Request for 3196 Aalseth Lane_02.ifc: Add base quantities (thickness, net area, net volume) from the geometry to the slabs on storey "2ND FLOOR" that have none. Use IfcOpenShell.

First a look at what the model holds.

```python
import ifcopenshell
import ifcopenshell.util.element
import ifcopenshell.util.unit

model = ifcopenshell.open("3196 Aalseth Lane_02.ifc")
print(model.schema)
for unit_type in ("LENGTHUNIT", "AREAUNIT", "VOLUMEUNIT"):
    print(unit_type, ifcopenshell.util.unit.calculate_unit_scale(model, unit_type))
storey = next(s for s in model.by_type("IfcBuildingStorey") if s.Name == "2ND FLOOR")
slabs = [e for e in ifcopenshell.util.element.get_decomposition(storey) if e.is_a("IfcSlab")]
for e in sorted(slabs, key=lambda e: e.id()):
    print(e.id(), e.is_a(), e.Name, list(ifcopenshell.util.element.get_psets(e, qtos_only=True)), sep=" | ")
```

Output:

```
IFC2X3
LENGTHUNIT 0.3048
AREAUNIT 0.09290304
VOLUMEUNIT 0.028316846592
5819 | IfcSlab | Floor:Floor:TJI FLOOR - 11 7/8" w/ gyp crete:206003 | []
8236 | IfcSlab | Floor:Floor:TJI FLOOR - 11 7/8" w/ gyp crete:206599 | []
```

```python
import ifcopenshell
import ifcopenshell.api.pset
import ifcopenshell.geom
import ifcopenshell.util.element
import ifcopenshell.util.shape
import ifcopenshell.util.unit

model = ifcopenshell.open("3196 Aalseth Lane_02.ifc")
unit_scale = ifcopenshell.util.unit.calculate_unit_scale(model)
area_scale = ifcopenshell.util.unit.calculate_unit_scale(model, "AREAUNIT")
volume_scale = ifcopenshell.util.unit.calculate_unit_scale(model, "VOLUMEUNIT")
settings = ifcopenshell.geom.settings()

storey = next(s for s in model.by_type("IfcBuildingStorey") if s.Name == "2ND FLOOR")
slabs = [e for e in ifcopenshell.util.element.get_decomposition(storey) if e.is_a("IfcSlab")]

for e in sorted(slabs, key=lambda e: e.id()):
    if ifcopenshell.util.element.get_psets(e, qtos_only=True, should_inherit=False):
        continue
    # Geometry comes back in metres, in the element's own axes.
    shape = ifcopenshell.geom.create_shape(settings, e)
    values = {
        "Width": ifcopenshell.util.shape.get_z(shape.geometry) / unit_scale,
        "NetArea": ifcopenshell.util.shape.get_footprint_area(shape.geometry) / area_scale,
        "NetVolume": ifcopenshell.util.shape.get_volume(shape.geometry) / volume_scale,
    }
    qto = ifcopenshell.api.pset.add_qto(model, product=e, name="BaseQuantities")
    ifcopenshell.api.pset.edit_qto(model, qto=qto, properties=values)
    print(e.id(), {k: round(v, 3) for k, v in values.items()})

model.write("3196 Aalseth Lane_02_v2.ifc")
```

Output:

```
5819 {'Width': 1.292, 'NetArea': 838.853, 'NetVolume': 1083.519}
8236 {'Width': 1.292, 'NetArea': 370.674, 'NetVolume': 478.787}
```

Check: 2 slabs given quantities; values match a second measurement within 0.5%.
